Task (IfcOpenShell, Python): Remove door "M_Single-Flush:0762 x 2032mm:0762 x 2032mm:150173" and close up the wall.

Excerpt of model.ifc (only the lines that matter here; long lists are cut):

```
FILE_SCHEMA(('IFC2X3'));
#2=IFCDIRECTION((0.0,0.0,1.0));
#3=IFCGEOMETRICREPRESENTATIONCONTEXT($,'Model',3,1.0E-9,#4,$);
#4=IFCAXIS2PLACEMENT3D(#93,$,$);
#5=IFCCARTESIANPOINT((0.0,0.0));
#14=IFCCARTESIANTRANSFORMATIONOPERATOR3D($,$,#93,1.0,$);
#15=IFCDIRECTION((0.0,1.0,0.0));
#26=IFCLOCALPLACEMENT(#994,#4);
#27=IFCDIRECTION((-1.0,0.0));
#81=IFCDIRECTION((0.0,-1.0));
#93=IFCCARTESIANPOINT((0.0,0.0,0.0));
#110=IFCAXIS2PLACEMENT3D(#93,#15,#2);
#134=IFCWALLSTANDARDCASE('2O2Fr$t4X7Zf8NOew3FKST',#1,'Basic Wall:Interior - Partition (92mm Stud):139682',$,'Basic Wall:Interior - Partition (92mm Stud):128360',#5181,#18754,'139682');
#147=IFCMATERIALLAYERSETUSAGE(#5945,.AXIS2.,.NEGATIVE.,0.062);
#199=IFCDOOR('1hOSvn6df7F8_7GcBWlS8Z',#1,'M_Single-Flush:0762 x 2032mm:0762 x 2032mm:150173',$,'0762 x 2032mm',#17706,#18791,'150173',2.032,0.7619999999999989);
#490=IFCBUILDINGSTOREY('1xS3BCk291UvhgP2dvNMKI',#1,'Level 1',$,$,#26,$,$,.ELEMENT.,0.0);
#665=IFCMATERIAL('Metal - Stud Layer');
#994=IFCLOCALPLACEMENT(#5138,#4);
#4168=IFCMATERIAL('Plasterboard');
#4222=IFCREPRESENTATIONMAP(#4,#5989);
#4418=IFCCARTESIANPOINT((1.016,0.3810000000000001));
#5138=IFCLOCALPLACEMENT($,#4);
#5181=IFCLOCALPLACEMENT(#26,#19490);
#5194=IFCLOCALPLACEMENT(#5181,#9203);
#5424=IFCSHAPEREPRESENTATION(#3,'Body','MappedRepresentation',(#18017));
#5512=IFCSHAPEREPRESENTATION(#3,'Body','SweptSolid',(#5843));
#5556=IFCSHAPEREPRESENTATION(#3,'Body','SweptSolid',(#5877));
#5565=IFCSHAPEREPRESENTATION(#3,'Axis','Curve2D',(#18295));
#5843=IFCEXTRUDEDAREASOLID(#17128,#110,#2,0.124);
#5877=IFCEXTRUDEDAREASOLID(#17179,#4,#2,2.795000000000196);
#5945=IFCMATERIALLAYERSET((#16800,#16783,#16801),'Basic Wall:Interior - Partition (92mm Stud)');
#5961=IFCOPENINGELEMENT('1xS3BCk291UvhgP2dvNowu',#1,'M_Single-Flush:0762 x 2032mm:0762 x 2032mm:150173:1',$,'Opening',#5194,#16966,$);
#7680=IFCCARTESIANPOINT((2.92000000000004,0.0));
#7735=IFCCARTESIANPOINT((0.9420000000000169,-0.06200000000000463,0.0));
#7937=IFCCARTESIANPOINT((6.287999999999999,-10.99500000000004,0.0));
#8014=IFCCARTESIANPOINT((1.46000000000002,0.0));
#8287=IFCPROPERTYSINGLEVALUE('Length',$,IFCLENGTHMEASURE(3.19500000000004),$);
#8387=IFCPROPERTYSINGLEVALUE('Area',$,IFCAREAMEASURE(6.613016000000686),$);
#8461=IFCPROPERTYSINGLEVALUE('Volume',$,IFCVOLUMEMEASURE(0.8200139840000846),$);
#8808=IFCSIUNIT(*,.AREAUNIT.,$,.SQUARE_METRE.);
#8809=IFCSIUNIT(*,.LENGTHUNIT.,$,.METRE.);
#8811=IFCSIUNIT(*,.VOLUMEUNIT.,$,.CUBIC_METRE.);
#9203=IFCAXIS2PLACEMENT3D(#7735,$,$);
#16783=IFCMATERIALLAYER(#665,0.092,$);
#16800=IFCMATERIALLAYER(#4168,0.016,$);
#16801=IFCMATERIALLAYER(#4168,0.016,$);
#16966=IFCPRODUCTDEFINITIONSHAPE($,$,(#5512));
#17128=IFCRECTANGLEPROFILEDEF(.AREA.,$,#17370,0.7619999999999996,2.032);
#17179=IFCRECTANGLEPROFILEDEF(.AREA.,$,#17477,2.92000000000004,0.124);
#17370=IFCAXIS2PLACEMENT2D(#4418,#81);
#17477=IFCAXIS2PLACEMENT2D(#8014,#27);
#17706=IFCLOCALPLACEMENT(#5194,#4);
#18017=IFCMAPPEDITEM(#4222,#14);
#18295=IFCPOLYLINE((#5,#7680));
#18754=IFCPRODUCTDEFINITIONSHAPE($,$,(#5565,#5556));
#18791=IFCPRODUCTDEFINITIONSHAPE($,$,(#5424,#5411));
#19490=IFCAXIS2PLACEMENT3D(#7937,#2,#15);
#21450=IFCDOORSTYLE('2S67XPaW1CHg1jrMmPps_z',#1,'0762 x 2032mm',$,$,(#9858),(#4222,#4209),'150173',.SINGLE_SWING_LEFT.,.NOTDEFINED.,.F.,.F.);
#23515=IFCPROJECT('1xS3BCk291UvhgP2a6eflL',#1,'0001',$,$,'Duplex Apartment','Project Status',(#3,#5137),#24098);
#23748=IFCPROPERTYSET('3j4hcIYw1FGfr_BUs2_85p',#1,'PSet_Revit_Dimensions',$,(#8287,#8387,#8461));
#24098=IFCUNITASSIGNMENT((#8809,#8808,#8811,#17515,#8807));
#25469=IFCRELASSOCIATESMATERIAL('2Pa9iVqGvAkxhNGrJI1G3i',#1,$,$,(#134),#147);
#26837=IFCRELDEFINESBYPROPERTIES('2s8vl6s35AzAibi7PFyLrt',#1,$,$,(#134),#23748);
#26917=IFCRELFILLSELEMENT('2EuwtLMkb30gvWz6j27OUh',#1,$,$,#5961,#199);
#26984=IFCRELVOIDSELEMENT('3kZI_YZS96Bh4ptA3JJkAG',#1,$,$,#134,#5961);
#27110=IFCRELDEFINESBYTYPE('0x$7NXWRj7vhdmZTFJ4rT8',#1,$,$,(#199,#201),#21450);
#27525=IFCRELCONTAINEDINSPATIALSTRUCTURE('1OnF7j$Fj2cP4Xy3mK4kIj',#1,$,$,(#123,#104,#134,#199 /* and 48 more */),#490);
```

```python
import ifcopenshell
import ifcopenshell.api.feature
import ifcopenshell.api.pset
import ifcopenshell.api.root
import ifcopenshell.geom
import ifcopenshell.util.element
import ifcopenshell.util.shape
import ifcopenshell.util.unit

model = ifcopenshell.open("model.ifc")
area_scale = ifcopenshell.util.unit.calculate_unit_scale(model, "AREAUNIT")
volume_scale = ifcopenshell.util.unit.calculate_unit_scale(model, "VOLUMEUNIT")
settings = ifcopenshell.geom.settings()


def volume(element):
    """Net volume in cubic metres, openings subtracted."""
    shape = ifcopenshell.geom.create_shape(settings, element)
    return ifcopenshell.util.shape.get_volume(shape.geometry)


door = model.by_guid("1hOSvn6df7F8_7GcBWlS8Z")
opening = door.FillsVoids[0].RelatingOpeningElement
wall = opening.VoidsElements[0].RelatingBuildingElement
before = volume(wall)

ifcopenshell.api.root.remove_product(model, product=door)
ifcopenshell.api.feature.remove_feature(model, feature=opening)

after = volume(wall)
thickness = 0.124  # wall thickness in metres

# Update the wall's stored quantities.
pset = model.by_id(ifcopenshell.util.element.get_pset(wall, "PSet_Revit_Dimensions", should_inherit=False)["id"])
ifcopenshell.api.pset.edit_pset(model, pset=pset, properties={
    "Area": model.create_entity("IfcAreaMeasure", after / thickness / area_scale),
    "Volume": model.create_entity("IfcVolumeMeasure", after / volume_scale),
})

print(f"wall volume {before:.3f} -> {after:.3f} m3")

model.write("model_edited.ifc")
```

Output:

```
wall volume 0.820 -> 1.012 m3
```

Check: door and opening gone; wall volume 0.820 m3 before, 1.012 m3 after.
